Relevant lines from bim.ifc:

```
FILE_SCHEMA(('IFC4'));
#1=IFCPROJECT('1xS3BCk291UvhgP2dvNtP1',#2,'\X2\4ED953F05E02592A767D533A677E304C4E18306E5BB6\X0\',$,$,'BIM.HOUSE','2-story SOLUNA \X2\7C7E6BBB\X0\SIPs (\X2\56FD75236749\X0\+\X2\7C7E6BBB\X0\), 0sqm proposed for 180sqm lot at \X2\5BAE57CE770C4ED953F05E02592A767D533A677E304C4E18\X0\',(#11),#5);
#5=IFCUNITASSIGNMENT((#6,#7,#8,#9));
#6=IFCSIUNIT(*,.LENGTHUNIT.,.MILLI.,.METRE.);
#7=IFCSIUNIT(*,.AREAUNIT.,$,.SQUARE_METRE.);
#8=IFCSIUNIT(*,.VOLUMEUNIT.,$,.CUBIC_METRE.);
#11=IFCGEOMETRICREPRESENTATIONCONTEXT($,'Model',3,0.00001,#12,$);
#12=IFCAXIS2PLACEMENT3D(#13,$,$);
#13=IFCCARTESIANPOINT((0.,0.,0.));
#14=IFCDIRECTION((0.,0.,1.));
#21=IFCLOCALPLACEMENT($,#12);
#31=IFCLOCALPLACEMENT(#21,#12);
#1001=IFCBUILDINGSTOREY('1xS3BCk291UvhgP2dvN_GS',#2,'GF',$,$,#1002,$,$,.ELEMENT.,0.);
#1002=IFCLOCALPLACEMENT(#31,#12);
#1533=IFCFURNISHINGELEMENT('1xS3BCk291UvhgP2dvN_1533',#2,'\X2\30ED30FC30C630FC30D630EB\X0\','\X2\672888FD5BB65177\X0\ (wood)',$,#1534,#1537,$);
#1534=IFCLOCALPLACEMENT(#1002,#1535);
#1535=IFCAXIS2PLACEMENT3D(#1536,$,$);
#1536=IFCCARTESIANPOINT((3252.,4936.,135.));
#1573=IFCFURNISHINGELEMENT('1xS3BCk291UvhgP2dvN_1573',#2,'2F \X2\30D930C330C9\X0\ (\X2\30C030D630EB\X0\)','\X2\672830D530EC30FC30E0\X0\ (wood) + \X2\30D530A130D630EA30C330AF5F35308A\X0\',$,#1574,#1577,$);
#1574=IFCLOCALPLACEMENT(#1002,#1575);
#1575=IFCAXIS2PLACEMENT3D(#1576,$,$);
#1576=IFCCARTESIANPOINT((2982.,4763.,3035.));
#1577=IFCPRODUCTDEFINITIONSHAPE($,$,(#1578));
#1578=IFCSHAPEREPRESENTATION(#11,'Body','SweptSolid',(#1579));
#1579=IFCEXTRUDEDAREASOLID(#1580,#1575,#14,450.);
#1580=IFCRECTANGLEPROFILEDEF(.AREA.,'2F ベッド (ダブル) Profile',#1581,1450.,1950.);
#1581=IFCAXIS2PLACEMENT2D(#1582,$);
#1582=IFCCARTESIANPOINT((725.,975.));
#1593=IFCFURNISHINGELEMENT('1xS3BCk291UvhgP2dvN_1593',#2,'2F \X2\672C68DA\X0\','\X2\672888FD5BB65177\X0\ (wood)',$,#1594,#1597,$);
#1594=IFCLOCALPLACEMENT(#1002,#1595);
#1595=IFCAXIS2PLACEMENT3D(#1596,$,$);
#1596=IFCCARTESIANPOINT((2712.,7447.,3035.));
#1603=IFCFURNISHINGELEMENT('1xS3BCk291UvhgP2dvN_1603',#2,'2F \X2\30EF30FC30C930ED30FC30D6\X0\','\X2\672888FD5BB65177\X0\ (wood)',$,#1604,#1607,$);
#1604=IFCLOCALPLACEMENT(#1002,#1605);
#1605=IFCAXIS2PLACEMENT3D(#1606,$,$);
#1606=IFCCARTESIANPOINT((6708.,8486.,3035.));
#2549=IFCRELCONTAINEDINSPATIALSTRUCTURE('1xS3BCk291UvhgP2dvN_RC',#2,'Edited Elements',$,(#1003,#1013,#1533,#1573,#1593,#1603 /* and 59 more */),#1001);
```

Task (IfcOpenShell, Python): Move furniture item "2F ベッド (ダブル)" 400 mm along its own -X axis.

```python
import ifcopenshell
import ifcopenshell.api.geometry
import ifcopenshell.util.placement

model = ifcopenshell.open("bim.ifc")

item = model.by_id(1573)
matrix = ifcopenshell.util.placement.get_local_placement(item.ObjectPlacement)
matrix[:3, 3] -= matrix[:3, 0] * 400.0
ifcopenshell.api.geometry.edit_object_placement(model, product=item, matrix=matrix, is_si=False)

print(ifcopenshell.util.placement.get_local_placement(item.ObjectPlacement).round(3) + 0.0)

model.write("bim_edited.ifc")
```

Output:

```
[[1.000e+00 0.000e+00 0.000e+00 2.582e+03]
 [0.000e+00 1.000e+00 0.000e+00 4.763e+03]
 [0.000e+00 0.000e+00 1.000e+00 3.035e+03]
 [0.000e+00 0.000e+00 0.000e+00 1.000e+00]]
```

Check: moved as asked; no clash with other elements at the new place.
